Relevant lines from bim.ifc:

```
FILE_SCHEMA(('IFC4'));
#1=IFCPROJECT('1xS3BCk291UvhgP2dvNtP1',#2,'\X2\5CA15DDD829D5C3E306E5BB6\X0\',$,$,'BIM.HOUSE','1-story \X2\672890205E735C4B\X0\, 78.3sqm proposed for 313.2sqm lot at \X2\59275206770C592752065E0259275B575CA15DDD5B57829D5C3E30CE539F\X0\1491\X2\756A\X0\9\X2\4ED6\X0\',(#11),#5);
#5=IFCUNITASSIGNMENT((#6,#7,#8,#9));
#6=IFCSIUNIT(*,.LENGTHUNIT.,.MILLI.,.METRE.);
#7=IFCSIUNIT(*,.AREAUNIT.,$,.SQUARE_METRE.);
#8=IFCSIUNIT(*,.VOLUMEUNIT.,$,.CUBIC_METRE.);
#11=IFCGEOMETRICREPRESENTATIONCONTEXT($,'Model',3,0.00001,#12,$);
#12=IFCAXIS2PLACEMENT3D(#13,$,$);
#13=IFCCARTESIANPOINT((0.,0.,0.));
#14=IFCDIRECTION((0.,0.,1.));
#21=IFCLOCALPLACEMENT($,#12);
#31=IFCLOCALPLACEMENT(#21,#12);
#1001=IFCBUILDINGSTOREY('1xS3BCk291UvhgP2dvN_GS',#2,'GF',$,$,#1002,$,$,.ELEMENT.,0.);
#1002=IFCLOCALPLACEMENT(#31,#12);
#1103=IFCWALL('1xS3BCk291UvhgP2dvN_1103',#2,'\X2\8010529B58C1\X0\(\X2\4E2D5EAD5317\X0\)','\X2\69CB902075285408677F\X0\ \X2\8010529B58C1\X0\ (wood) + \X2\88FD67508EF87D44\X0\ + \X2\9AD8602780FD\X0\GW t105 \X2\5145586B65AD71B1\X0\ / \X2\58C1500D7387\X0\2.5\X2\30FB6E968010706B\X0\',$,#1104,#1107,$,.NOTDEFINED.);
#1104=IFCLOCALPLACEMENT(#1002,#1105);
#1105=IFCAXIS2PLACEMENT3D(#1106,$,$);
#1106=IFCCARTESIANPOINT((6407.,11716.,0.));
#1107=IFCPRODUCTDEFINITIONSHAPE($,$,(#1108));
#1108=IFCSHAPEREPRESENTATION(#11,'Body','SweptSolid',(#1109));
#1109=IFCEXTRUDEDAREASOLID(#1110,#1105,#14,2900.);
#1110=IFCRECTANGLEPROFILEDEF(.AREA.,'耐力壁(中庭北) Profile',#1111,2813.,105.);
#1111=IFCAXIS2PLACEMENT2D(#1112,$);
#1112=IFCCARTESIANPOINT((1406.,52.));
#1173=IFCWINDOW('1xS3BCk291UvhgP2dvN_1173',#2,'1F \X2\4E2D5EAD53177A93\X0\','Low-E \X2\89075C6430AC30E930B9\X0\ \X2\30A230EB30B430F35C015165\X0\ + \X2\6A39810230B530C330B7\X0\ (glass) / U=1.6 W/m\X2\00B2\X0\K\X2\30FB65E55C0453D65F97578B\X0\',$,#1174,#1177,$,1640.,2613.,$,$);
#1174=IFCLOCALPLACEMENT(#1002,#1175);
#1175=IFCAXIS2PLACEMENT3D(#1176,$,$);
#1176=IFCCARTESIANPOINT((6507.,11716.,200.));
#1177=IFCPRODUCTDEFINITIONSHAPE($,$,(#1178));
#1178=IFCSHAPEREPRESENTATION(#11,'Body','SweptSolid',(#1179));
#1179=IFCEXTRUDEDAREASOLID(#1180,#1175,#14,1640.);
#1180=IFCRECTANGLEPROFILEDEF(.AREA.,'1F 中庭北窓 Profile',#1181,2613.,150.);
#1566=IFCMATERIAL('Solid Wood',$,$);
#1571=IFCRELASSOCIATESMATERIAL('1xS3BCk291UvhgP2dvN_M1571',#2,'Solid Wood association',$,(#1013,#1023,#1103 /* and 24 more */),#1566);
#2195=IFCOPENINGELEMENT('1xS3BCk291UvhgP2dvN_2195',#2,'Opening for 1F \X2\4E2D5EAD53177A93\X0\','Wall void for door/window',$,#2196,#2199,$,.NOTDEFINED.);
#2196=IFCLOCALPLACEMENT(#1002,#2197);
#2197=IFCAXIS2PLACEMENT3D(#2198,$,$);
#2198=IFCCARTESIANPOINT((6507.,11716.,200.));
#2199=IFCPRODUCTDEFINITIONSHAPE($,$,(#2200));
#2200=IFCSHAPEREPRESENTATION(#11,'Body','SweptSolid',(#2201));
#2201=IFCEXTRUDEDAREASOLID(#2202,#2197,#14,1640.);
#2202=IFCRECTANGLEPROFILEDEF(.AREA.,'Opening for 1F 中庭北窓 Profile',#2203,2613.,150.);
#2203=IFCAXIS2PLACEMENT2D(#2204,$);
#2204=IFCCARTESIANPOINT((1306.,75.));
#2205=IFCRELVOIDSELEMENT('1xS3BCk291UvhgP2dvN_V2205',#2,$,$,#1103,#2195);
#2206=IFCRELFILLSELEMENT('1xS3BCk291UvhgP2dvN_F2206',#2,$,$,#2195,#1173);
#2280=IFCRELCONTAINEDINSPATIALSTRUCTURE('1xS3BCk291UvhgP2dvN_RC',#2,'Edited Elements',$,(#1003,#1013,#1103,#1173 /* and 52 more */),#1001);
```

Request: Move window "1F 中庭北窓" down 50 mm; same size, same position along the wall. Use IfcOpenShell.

```python
import numpy as np
import ifcopenshell
import ifcopenshell.api.geometry
import ifcopenshell.util.placement
import ifcopenshell.util.unit

model = ifcopenshell.open("bim.ifc")
unit_scale = ifcopenshell.util.unit.calculate_unit_scale(model)

window = model.by_id(1173)
opening = window.FillsVoids[0].RelatingOpeningElement
dz = -0.05 / unit_scale

shift = np.array([0.0, 0.0, dz])
# The window is not placed relative to its opening, so move both.
for product in (opening, window):
    matrix = ifcopenshell.util.placement.get_local_placement(product.ObjectPlacement)
    matrix[:3, 3] += shift
    ifcopenshell.api.geometry.edit_object_placement(model, product=product, matrix=matrix, is_si=False)

print(f"moved by {dz * unit_scale:+.3f} m")

model.write("bim-out.ifc")
```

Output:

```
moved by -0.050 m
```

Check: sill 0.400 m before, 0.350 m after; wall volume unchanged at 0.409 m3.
